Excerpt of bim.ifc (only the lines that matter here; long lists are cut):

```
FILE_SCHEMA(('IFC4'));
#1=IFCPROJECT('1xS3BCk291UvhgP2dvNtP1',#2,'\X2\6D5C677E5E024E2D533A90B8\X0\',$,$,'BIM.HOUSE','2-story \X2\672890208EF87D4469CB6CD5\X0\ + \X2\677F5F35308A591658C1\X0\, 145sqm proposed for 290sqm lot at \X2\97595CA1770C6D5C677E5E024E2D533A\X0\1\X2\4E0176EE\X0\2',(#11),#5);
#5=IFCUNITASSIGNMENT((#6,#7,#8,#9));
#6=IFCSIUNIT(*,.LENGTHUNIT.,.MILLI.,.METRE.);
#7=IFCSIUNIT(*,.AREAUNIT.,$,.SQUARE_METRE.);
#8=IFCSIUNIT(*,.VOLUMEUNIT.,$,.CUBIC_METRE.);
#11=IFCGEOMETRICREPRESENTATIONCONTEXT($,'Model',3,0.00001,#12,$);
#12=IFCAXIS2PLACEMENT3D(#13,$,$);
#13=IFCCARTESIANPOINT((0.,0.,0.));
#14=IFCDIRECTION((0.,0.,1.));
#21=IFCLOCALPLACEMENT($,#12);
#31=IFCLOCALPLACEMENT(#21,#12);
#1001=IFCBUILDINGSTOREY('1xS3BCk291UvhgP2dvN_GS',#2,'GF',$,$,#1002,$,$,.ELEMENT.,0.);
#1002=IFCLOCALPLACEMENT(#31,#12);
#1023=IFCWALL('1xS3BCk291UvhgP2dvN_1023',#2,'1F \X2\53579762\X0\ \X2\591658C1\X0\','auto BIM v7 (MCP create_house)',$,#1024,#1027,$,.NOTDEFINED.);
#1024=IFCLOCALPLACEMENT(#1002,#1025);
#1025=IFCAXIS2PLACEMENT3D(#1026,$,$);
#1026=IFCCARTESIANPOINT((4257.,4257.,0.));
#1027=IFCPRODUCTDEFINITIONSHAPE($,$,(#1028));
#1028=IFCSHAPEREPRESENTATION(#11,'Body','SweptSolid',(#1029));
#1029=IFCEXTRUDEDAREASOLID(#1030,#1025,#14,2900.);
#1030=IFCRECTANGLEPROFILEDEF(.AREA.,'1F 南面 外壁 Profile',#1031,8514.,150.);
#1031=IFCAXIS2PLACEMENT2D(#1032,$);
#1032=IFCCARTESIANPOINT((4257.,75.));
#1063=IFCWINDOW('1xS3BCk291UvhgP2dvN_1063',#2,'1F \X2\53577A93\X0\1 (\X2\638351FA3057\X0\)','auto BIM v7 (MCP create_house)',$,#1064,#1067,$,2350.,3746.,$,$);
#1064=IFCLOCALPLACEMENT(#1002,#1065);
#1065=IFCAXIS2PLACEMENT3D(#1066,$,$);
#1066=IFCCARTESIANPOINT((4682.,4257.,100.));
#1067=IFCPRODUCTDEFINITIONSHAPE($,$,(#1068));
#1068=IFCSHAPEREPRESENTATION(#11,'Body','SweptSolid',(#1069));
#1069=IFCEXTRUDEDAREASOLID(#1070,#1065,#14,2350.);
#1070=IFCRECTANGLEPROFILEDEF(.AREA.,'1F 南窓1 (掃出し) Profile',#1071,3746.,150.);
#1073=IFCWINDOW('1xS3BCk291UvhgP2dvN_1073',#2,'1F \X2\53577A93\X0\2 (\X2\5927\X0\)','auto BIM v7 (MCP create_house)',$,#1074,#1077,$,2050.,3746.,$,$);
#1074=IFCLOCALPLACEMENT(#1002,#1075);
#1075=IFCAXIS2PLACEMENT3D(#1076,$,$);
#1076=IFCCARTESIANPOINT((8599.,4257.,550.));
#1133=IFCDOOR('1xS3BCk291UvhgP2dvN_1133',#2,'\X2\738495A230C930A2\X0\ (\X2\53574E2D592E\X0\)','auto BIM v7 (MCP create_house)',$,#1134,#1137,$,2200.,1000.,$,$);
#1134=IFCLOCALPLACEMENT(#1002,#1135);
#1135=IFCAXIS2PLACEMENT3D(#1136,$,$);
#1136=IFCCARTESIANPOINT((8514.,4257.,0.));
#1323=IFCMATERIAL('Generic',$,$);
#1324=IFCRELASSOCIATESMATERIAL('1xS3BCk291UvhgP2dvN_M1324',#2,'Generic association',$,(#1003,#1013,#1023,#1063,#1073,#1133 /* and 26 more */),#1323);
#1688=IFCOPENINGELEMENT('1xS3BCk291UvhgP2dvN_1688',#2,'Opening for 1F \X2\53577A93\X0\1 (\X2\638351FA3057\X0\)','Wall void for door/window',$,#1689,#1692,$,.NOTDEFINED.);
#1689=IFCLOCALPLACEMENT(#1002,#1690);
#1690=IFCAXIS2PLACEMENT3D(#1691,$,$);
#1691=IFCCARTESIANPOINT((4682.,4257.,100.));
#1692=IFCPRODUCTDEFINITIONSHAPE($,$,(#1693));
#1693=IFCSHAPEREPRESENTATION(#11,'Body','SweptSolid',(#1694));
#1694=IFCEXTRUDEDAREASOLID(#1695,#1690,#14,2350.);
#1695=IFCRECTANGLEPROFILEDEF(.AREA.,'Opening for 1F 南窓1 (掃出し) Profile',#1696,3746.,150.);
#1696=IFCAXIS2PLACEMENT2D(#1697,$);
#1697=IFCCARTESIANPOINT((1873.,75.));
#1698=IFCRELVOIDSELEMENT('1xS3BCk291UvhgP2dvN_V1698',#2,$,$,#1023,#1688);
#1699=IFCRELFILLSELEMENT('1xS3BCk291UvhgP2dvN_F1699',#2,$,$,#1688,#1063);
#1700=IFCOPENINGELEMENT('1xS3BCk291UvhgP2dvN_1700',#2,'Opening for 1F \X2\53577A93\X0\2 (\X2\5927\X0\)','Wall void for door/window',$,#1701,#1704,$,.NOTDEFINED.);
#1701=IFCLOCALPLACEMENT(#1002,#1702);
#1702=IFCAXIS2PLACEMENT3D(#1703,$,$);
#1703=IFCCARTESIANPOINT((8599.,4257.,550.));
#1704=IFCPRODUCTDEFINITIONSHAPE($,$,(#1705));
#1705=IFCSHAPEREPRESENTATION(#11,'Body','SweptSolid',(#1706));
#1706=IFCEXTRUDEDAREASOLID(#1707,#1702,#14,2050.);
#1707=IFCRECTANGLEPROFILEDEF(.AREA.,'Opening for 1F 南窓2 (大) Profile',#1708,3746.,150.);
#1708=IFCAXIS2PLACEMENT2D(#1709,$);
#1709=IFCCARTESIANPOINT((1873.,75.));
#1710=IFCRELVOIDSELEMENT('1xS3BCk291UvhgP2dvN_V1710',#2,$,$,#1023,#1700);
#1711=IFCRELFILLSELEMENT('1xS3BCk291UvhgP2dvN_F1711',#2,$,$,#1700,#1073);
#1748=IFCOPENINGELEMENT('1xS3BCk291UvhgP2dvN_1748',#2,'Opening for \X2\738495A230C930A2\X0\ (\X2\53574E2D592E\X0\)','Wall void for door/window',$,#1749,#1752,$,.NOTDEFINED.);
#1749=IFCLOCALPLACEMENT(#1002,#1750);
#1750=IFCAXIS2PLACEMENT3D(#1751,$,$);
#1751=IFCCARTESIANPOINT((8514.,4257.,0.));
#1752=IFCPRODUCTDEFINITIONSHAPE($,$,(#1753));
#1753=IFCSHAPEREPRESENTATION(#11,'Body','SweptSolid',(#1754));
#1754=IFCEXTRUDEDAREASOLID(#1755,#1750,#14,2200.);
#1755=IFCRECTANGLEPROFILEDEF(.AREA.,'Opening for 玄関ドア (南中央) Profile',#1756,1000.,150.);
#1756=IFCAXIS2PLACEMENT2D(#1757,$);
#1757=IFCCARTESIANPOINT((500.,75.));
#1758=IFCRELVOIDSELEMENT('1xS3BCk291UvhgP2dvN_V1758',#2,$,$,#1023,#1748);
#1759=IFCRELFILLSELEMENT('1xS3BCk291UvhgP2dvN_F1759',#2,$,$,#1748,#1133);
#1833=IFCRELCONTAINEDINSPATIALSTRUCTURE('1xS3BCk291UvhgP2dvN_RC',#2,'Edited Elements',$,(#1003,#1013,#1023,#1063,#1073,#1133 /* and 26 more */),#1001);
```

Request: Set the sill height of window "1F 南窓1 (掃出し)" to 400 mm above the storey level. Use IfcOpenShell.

```python
import numpy as np
import ifcopenshell
import ifcopenshell.api.geometry
import ifcopenshell.geom
import ifcopenshell.util.element
import ifcopenshell.util.placement
import ifcopenshell.util.shape
import ifcopenshell.util.unit

model = ifcopenshell.open("bim.ifc")
unit_scale = ifcopenshell.util.unit.calculate_unit_scale(model)

window = model.by_guid("1xS3BCk291UvhgP2dvN_1063")
opening = window.FillsVoids[0].RelatingOpeningElement
storey = ifcopenshell.util.element.get_container(window, ifc_class="IfcBuildingStorey")
level = ifcopenshell.util.placement.get_local_placement(storey.ObjectPlacement)[2, 3]

# The opening's origin need not be at the sill, so measure its lowest point.
shape = ifcopenshell.geom.create_shape(ifcopenshell.geom.settings(), opening)
bottom = ifcopenshell.util.shape.get_shape_bottom_elevation(shape, shape.geometry) / unit_scale
dz = level + 0.4 / unit_scale - bottom

shift = np.array([0.0, 0.0, dz])
# The window is not placed relative to its opening, so move both.
for product in (opening, window):
    matrix = ifcopenshell.util.placement.get_local_placement(product.ObjectPlacement)
    matrix[:3, 3] += shift
    ifcopenshell.api.geometry.edit_object_placement(model, product=product, matrix=matrix, is_si=False)

print(f"moved by {dz * unit_scale:+.3f} m")

model.write("bim_v2.ifc")
```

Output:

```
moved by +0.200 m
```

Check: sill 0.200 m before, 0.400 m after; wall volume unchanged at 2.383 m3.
